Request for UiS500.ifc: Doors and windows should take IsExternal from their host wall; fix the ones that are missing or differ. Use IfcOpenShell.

First a look at what the model holds.

```python
import ifcopenshell
import ifcopenshell.util.element

model = ifcopenshell.open("UiS500.ifc")
print(model.schema)
seen = {}
for e in model.by_type("IfcDoor") + model.by_type("IfcWindow"):
    if not e.FillsVoids:
        continue
    host = e.FillsVoids[0].RelatingOpeningElement.VoidsElements[0].RelatingBuildingElement
    own = ifcopenshell.util.element.get_pset(e, f"Pset_{e.is_a()[3:].removesuffix('StandardCase')}Common", "IsExternal")
    wall = ifcopenshell.util.element.get_pset(host, "Pset_WallCommon", "IsExternal")
    seen[e.is_a(), own, wall] = seen.get((e.is_a(), own, wall), 0) + 1
for (cls, own, wall), count in sorted(seen.items(), key=str):
    print(count, cls, "IsExternal:", own, "| host wall:", wall)
```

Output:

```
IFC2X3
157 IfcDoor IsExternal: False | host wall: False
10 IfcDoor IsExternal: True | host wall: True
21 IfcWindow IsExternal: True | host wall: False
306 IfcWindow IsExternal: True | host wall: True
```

```python
import ifcopenshell
import ifcopenshell.api.pset
import ifcopenshell.util.element

model = ifcopenshell.open("UiS500.ifc")

count = 0
for ifc_class, pset_name in (("IfcDoor", "Pset_DoorCommon"), ("IfcWindow", "Pset_WindowCommon")):
    for e in model.by_type(ifc_class):
        if not e.FillsVoids:
            continue
        host = e.FillsVoids[0].RelatingOpeningElement.VoidsElements[0].RelatingBuildingElement
        external = ifcopenshell.util.element.get_pset(host, "Pset_WallCommon", "IsExternal")
        if external is None or ifcopenshell.util.element.get_pset(e, pset_name, "IsExternal") == external:
            continue
        found = ifcopenshell.util.element.get_pset(e, pset_name, should_inherit=False)
        if found:
            pset = model.by_id(found["id"])
            if len(ifcopenshell.util.element.get_elements_by_pset(pset)) > 1:
                pset = ifcopenshell.api.pset.unshare_pset(model, products=[e], pset=pset)[0]
        else:
            pset = ifcopenshell.api.pset.add_pset(model, product=e, name=pset_name)
        ifcopenshell.api.pset.edit_pset(model, pset=pset, properties={"IsExternal": external})
        count += 1

print(count, "updated")

model.write("UiS500_v2.ifc")
```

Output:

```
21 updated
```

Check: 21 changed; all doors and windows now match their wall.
